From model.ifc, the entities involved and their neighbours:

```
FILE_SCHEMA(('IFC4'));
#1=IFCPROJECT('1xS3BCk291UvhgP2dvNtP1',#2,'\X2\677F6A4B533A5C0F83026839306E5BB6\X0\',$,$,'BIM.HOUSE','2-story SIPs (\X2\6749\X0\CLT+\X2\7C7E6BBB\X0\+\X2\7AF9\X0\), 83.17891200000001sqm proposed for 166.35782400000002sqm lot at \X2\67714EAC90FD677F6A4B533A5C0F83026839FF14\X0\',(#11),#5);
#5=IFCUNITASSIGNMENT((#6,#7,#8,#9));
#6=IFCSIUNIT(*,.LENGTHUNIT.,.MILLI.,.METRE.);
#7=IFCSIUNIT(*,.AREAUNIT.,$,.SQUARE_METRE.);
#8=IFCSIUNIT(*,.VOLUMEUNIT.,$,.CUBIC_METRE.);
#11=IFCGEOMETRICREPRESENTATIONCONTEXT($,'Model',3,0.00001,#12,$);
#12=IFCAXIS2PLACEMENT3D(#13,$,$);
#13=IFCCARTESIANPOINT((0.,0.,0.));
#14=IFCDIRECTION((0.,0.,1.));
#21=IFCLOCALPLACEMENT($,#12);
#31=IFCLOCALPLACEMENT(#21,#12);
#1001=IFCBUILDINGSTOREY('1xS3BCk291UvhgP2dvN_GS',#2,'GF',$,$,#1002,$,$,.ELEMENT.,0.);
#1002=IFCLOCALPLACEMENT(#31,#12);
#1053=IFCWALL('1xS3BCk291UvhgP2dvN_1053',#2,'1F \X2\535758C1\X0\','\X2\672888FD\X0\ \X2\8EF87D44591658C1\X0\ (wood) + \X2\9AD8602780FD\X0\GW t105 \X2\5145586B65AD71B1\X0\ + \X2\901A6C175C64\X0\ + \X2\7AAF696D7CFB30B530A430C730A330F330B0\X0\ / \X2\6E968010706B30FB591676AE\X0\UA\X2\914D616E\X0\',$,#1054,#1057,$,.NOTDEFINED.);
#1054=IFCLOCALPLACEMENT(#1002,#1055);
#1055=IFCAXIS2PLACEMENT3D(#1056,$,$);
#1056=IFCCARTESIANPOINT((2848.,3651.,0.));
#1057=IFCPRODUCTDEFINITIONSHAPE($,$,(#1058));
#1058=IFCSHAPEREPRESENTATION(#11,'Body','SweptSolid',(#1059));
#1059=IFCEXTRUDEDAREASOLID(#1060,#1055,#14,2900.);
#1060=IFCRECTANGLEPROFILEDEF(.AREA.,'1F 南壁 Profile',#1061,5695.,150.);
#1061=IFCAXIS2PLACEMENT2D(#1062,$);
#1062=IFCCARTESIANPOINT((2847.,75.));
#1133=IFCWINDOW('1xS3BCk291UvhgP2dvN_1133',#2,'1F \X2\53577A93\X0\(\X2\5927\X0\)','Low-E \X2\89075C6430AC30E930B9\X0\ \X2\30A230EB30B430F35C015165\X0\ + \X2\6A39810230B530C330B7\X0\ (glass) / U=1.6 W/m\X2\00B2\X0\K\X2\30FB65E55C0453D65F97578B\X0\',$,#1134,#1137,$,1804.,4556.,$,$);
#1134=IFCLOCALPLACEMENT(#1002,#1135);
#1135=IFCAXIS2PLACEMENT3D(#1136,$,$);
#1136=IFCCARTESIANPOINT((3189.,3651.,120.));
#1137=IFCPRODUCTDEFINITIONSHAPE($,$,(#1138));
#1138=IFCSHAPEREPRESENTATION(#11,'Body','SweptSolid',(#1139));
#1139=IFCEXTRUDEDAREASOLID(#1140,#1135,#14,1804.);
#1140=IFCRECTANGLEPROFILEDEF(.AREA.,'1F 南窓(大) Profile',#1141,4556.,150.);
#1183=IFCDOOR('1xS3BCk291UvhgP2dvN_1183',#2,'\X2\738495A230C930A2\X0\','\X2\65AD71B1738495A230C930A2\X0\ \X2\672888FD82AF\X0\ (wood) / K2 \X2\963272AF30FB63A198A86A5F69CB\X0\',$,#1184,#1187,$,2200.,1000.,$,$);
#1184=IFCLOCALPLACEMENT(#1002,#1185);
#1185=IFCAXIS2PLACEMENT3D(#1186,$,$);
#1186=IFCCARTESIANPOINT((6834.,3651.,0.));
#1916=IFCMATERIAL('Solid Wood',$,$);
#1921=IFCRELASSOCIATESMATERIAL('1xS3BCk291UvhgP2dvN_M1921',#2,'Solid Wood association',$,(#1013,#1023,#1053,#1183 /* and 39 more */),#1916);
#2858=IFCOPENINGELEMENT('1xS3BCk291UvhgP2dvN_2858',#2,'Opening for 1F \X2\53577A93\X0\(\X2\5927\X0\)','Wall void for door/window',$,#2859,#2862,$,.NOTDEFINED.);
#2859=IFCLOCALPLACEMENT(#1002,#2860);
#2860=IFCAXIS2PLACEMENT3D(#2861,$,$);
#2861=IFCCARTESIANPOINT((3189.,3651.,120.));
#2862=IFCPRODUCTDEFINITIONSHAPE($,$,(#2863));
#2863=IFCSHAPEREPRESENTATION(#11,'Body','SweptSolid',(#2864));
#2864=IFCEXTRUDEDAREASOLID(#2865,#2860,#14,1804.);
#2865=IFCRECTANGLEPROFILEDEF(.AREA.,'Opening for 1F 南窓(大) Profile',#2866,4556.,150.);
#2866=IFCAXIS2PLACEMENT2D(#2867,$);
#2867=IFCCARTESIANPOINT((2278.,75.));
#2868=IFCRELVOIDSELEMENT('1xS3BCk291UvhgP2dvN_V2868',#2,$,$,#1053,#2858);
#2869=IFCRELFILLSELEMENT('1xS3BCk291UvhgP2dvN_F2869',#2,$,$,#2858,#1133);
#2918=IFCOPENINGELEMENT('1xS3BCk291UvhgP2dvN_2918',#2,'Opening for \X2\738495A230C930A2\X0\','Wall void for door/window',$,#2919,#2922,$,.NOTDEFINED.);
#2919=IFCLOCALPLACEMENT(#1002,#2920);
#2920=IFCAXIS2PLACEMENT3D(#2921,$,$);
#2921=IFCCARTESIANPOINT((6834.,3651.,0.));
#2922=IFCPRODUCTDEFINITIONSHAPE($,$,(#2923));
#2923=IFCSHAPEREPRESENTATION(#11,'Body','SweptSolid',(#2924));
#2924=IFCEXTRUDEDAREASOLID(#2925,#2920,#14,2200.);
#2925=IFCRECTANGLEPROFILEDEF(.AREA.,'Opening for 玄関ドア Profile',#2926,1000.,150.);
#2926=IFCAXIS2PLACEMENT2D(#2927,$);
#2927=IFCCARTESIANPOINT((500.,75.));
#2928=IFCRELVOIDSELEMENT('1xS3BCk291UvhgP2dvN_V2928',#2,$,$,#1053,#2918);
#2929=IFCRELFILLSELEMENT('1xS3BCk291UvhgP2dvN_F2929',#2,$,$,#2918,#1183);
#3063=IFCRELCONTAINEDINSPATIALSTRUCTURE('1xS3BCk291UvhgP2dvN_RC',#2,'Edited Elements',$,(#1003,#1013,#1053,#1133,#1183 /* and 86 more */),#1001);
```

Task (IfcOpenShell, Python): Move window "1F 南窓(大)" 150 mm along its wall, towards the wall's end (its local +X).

```python
import ifcopenshell
import ifcopenshell.api.geometry
import ifcopenshell.util.placement
import ifcopenshell.util.unit

model = ifcopenshell.open("model.ifc")
unit_scale = ifcopenshell.util.unit.calculate_unit_scale(model)

window = model.by_id(1133)
opening = window.FillsVoids[0].RelatingOpeningElement
wall = opening.VoidsElements[0].RelatingBuildingElement

wall_matrix = ifcopenshell.util.placement.get_local_placement(wall.ObjectPlacement)
shift = wall_matrix[:3, 0] * 0.15 / unit_scale
before = ifcopenshell.util.placement.get_local_placement(window.ObjectPlacement)[:3, 3].copy()

# The window is not placed relative to its opening, so move both.
for product in (opening, window):
    matrix = ifcopenshell.util.placement.get_local_placement(product.ObjectPlacement)
    matrix[:3, 3] += shift
    ifcopenshell.api.geometry.edit_object_placement(model, product=product, matrix=matrix, is_si=False)

after = ifcopenshell.util.placement.get_local_placement(window.ObjectPlacement)[:3, 3]
print("window moved by", (after - before).round(3) + 0.0)

model.write("model_v2.ifc")
```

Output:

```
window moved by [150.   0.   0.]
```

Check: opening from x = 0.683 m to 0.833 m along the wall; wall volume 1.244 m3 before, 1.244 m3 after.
